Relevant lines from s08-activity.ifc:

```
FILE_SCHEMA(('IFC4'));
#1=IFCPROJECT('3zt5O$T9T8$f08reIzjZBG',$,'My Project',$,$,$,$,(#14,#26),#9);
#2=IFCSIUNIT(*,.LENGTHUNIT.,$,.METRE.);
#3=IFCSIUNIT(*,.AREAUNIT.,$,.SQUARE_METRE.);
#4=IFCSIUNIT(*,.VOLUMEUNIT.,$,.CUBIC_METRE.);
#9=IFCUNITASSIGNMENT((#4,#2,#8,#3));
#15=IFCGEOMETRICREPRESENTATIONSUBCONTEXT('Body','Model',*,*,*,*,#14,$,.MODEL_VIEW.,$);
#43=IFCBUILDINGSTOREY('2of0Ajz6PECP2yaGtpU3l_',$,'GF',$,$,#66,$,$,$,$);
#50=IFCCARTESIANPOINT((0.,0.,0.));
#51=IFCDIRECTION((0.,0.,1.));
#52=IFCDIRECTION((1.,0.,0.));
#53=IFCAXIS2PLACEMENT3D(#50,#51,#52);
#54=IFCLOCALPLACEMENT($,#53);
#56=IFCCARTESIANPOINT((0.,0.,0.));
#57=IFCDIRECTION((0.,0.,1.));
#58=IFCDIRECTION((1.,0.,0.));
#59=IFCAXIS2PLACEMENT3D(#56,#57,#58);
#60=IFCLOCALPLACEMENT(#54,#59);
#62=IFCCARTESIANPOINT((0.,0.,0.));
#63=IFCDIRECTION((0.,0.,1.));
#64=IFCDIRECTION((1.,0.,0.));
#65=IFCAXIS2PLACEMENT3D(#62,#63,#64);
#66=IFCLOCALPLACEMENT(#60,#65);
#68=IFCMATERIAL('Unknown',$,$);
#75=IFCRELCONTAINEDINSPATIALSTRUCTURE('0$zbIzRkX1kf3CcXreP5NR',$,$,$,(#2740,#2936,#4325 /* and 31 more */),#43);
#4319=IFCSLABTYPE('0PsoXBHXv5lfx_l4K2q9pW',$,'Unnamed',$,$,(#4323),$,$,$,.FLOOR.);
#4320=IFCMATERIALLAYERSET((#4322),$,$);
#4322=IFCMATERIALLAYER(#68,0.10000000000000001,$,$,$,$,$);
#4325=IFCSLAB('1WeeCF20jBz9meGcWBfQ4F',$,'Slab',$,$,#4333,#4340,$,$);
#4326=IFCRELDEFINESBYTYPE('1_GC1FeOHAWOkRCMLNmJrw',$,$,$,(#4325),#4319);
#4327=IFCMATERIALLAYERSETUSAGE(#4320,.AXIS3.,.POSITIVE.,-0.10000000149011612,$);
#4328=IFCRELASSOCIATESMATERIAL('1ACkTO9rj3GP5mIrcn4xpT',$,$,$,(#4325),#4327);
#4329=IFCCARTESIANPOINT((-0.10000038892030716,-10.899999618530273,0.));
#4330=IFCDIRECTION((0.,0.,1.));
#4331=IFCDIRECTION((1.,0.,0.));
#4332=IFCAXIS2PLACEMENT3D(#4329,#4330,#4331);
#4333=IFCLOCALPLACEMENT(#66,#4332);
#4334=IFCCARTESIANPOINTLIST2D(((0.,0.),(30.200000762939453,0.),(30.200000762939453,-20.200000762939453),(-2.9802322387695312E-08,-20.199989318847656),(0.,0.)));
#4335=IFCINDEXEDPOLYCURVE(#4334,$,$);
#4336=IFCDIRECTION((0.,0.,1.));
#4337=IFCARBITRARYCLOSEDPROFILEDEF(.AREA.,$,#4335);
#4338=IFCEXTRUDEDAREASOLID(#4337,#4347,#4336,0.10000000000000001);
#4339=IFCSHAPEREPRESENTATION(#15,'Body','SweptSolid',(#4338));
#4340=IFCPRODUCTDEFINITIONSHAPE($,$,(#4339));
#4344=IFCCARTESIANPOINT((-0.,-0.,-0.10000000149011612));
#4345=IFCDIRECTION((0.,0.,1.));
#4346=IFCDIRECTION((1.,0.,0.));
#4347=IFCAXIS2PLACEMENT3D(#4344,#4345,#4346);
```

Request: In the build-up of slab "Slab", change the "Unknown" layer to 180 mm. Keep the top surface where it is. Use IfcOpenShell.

```python
import ifcopenshell
import ifcopenshell.util.element
import ifcopenshell.util.representation

model = ifcopenshell.open("s08-activity.ifc")

layer_set = model.by_id(4320)
layer = next(l for l in layer_set.MaterialLayers if l.Material and l.Material.Name == "Unknown")
change = 0.18 - layer.LayerThickness
layer.LayerThickness += change

# Geometry does not follow the layer set by itself.
slabs = [e for e in ifcopenshell.util.element.get_elements_by_material(model, layer_set) if e.is_a("IfcSlab")]
for slab in sorted(slabs, key=lambda e: e.id()):
    body = ifcopenshell.util.representation.get_representation(slab, "Model", "Body")
    solid = body.Items[0]
    old_depth = solid.Depth
    solid.Depth += change
    # Extruded upwards: lower the start of the extrusion so the top stays.
    x, y, z = solid.Position.Location.Coordinates
    solid.Position.Location = model.createIfcCartesianPoint((x, y, z - change))
    print(slab.id(), f"{old_depth:g} -> {solid.Depth:g}")

# The layers are counted up from the underside, which has moved.
for usage in {ifcopenshell.util.element.get_material(slab) for slab in slabs}:
    usage.OffsetFromReferenceLine -= change

model.write("s08-activity_v2.ifc")
```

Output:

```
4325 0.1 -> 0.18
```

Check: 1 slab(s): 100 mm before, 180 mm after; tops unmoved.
